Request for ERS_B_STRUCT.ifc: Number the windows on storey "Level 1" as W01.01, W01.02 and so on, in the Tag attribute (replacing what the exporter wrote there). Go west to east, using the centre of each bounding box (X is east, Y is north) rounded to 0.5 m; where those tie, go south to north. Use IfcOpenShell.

First a look at what the model holds.

```python
import ifcopenshell
import ifcopenshell.util.element
import ifcopenshell.util.placement

model = ifcopenshell.open("ERS_B_STRUCT.ifc")
print(model.schema)
storey = next(s for s in model.by_type("IfcBuildingStorey") if s.Name == "Level 1")
windows = [e for e in ifcopenshell.util.element.get_decomposition(storey) if e.is_a("IfcWindow")]
for e in sorted(windows, key=lambda e: e.id()):
    origin = ifcopenshell.util.placement.get_local_placement(e.ObjectPlacement)[:3, 3]
    print(e.id(), e.Tag, e.Name, origin.round(2) + 0.0, sep=" | ")
```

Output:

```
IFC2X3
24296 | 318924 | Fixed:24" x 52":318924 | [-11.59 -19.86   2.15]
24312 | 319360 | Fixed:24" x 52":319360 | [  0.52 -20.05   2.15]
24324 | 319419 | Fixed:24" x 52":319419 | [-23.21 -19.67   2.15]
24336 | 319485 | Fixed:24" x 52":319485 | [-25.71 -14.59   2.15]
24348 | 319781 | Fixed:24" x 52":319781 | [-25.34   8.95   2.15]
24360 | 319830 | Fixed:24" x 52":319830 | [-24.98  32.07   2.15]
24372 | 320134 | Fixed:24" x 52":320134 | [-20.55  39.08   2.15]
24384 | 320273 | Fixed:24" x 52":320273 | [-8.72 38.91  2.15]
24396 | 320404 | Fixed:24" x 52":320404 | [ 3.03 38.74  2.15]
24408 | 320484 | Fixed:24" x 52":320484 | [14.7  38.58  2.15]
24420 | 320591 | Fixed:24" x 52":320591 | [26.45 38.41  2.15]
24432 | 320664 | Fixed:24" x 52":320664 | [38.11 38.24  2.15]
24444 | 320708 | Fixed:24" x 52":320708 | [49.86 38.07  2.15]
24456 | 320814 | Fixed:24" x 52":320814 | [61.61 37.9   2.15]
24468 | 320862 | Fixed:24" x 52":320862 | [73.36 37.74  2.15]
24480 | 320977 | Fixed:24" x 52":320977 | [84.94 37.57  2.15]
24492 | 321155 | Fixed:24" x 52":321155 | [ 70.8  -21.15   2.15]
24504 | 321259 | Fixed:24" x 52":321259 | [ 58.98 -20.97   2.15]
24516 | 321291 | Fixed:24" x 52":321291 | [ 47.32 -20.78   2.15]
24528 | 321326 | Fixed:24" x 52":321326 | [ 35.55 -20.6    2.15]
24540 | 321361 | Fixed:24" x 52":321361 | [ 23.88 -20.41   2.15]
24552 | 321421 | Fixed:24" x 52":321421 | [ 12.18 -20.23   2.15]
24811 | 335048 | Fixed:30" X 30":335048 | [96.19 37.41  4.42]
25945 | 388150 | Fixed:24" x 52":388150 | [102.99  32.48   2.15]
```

```python
import ifcopenshell
import ifcopenshell.geom
import ifcopenshell.util.element
import ifcopenshell.util.shape

model = ifcopenshell.open("ERS_B_STRUCT.ifc")
settings = ifcopenshell.geom.settings()
settings.set("use-world-coords", True)


def centre(element):
    shape = ifcopenshell.geom.create_shape(settings, element)
    return ifcopenshell.util.shape.get_bbox_centroid(shape.geometry)


storey = next(s for s in model.by_type("IfcBuildingStorey") if s.Name == "Level 1")
windows = [e for e in ifcopenshell.util.element.get_decomposition(storey) if e.is_a("IfcWindow")]

# Insertion points can sit at a corner or the storey origin, so sort by the geometry (in metres).
centres = {e: centre(e) for e in windows}
windows.sort(key=lambda e: (round(centres[e][0] / 0.5), centres[e][1]))

for i, e in enumerate(windows, start=1):
    number = f"W01.{i:02d}"
    e.Tag = number
    print(e.id(), number)

model.write("ERS_B_STRUCT_v2.ifc")
```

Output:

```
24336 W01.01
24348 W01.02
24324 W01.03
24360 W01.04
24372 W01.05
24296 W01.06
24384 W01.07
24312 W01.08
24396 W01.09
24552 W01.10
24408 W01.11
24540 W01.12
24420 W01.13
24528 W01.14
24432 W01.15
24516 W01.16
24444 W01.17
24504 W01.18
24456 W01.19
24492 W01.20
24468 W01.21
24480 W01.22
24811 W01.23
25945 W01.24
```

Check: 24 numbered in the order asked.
